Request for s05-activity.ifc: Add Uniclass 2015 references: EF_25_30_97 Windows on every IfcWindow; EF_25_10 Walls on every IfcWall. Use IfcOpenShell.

First a look at what the model holds.

```python
import ifcopenshell

model = ifcopenshell.open("s05-activity.ifc")
print(model.schema)
print("classifications:", [c.Name for c in model.by_type("IfcClassification")])
for ifc_class in ("IfcDoor", "IfcRoof", "IfcStair", "IfcWall", "IfcWindow"):
    print(ifc_class, len(model.by_type(ifc_class)))
```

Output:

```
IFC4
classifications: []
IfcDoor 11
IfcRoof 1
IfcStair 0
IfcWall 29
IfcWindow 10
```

```python
import ifcopenshell
import ifcopenshell.api.classification

model = ifcopenshell.open("s05-activity.ifc")

system = ifcopenshell.api.classification.add_classification(model, classification="Uniclass 2015")

codes = {
    "IfcWindow": ("EF_25_30_97", "Windows"),
    "IfcWall": ("EF_25_10", "Walls"),
}
for ifc_class, (code, name) in codes.items():
    products = model.by_type(ifc_class)
    ifcopenshell.api.classification.add_reference(
        model, products=products, classification=system, identification=code, name=name
    )
    print(code, len(products))

model.write("s05-activity_rev.ifc")
```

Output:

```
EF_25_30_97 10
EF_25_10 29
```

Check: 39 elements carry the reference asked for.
